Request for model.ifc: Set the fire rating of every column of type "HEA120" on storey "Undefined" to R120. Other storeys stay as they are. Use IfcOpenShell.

First a look at what the model holds.

```python
import ifcopenshell
import ifcopenshell.util.element

model = ifcopenshell.open("model.ifc")
print(model.schema)
storey = next(s for s in model.by_type("IfcBuildingStorey") if s.Name == "Undefined")
columns = [e for e in ifcopenshell.util.element.get_decomposition(storey) if e.is_a("IfcColumn")]
seen = {}
for e in columns:
    element_type = ifcopenshell.util.element.get_type(e)
    key = (element_type.Name if element_type != e and element_type else None, ifcopenshell.util.element.get_pset(e, "Pset_ColumnCommon", "FireRating"))
    seen[key] = seen.get(key, 0) + 1
for (name, value), count in sorted(seen.items(), key=str):
    print(count, "x", name, "|", value)
```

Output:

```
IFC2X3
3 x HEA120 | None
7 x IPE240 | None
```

```python
import ifcopenshell
import ifcopenshell.api.pset
import ifcopenshell.util.element

model = ifcopenshell.open("model.ifc")

storey = next(s for s in model.by_type("IfcBuildingStorey") if s.Name == "Undefined")
columns = [e for e in ifcopenshell.util.element.get_decomposition(storey) if e.is_a("IfcColumn")]

count = 0
for e in columns:
    element_type = ifcopenshell.util.element.get_type(e)
    if element_type in (None, e) or element_type.Name != "HEA120":
        continue
    # add_pset returns the element's existing set when there is one.
    pset = ifcopenshell.api.pset.add_pset(model, product=e, name="Pset_ColumnCommon")
    ifcopenshell.api.pset.edit_pset(model, pset=pset, properties={"FireRating": "R120"})
    count += 1

print(count, "columns updated")

model.write("model_rev.ifc")
```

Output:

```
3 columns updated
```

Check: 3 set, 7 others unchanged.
